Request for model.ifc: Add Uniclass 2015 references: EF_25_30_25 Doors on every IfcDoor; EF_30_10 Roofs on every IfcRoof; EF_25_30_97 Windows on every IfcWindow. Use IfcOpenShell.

First a look at what the model holds.

```python
import ifcopenshell

model = ifcopenshell.open("model.ifc")
print(model.schema)
print("classifications:", [c.Name for c in model.by_type("IfcClassification")])
for ifc_class in ("IfcDoor", "IfcRoof", "IfcStair", "IfcWall", "IfcWindow"):
    print(ifc_class, len(model.by_type(ifc_class)))
```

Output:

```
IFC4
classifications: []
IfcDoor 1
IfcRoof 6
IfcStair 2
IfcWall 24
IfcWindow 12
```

```python
import ifcopenshell
import ifcopenshell.api.classification

model = ifcopenshell.open("model.ifc")

system = ifcopenshell.api.classification.add_classification(model, classification="Uniclass 2015")

codes = {
    "IfcDoor": ("EF_25_30_25", "Doors"),
    "IfcRoof": ("EF_30_10", "Roofs"),
    "IfcWindow": ("EF_25_30_97", "Windows"),
}
for ifc_class, (code, name) in codes.items():
    products = model.by_type(ifc_class)
    ifcopenshell.api.classification.add_reference(
        model, products=products, classification=system, identification=code, name=name
    )
    print(code, len(products))

model.write("model-out.ifc")
```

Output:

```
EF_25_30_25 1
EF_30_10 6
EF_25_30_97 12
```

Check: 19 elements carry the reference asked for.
